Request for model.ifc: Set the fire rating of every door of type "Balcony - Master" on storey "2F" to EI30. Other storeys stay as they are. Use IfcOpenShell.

First a look at what the model holds.

```python
import ifcopenshell
import ifcopenshell.util.element

model = ifcopenshell.open("model.ifc")
print(model.schema)
storey = next(s for s in model.by_type("IfcBuildingStorey") if s.Name == "2F")
doors = [e for e in ifcopenshell.util.element.get_decomposition(storey) if e.is_a("IfcDoor")]
seen = {}
for e in doors:
    element_type = ifcopenshell.util.element.get_type(e)
    key = (element_type.Name if element_type != e and element_type else None, ifcopenshell.util.element.get_pset(e, "Pset_DoorCommon", "FireRating"))
    seen[key] = seen.get(key, 0) + 1
for (name, value), count in sorted(seen.items(), key=str):
    print(count, "x", name, "|", value)
```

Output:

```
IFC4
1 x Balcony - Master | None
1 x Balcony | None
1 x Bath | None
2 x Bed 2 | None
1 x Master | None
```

```python
import ifcopenshell
import ifcopenshell.api.pset
import ifcopenshell.util.element

model = ifcopenshell.open("model.ifc")

storey = next(s for s in model.by_type("IfcBuildingStorey") if s.Name == "2F")
doors = [e for e in ifcopenshell.util.element.get_decomposition(storey) if e.is_a("IfcDoor")]

count = 0
for e in doors:
    element_type = ifcopenshell.util.element.get_type(e)
    if element_type in (None, e) or element_type.Name != "Balcony - Master":
        continue
    # add_pset returns the element's existing set when there is one.
    pset = ifcopenshell.api.pset.add_pset(model, product=e, name="Pset_DoorCommon")
    ifcopenshell.api.pset.edit_pset(model, pset=pset, properties={"FireRating": "EI30"})
    count += 1

print(count, "doors updated")

model.write("model_updated.ifc")
```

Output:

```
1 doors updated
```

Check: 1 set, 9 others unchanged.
